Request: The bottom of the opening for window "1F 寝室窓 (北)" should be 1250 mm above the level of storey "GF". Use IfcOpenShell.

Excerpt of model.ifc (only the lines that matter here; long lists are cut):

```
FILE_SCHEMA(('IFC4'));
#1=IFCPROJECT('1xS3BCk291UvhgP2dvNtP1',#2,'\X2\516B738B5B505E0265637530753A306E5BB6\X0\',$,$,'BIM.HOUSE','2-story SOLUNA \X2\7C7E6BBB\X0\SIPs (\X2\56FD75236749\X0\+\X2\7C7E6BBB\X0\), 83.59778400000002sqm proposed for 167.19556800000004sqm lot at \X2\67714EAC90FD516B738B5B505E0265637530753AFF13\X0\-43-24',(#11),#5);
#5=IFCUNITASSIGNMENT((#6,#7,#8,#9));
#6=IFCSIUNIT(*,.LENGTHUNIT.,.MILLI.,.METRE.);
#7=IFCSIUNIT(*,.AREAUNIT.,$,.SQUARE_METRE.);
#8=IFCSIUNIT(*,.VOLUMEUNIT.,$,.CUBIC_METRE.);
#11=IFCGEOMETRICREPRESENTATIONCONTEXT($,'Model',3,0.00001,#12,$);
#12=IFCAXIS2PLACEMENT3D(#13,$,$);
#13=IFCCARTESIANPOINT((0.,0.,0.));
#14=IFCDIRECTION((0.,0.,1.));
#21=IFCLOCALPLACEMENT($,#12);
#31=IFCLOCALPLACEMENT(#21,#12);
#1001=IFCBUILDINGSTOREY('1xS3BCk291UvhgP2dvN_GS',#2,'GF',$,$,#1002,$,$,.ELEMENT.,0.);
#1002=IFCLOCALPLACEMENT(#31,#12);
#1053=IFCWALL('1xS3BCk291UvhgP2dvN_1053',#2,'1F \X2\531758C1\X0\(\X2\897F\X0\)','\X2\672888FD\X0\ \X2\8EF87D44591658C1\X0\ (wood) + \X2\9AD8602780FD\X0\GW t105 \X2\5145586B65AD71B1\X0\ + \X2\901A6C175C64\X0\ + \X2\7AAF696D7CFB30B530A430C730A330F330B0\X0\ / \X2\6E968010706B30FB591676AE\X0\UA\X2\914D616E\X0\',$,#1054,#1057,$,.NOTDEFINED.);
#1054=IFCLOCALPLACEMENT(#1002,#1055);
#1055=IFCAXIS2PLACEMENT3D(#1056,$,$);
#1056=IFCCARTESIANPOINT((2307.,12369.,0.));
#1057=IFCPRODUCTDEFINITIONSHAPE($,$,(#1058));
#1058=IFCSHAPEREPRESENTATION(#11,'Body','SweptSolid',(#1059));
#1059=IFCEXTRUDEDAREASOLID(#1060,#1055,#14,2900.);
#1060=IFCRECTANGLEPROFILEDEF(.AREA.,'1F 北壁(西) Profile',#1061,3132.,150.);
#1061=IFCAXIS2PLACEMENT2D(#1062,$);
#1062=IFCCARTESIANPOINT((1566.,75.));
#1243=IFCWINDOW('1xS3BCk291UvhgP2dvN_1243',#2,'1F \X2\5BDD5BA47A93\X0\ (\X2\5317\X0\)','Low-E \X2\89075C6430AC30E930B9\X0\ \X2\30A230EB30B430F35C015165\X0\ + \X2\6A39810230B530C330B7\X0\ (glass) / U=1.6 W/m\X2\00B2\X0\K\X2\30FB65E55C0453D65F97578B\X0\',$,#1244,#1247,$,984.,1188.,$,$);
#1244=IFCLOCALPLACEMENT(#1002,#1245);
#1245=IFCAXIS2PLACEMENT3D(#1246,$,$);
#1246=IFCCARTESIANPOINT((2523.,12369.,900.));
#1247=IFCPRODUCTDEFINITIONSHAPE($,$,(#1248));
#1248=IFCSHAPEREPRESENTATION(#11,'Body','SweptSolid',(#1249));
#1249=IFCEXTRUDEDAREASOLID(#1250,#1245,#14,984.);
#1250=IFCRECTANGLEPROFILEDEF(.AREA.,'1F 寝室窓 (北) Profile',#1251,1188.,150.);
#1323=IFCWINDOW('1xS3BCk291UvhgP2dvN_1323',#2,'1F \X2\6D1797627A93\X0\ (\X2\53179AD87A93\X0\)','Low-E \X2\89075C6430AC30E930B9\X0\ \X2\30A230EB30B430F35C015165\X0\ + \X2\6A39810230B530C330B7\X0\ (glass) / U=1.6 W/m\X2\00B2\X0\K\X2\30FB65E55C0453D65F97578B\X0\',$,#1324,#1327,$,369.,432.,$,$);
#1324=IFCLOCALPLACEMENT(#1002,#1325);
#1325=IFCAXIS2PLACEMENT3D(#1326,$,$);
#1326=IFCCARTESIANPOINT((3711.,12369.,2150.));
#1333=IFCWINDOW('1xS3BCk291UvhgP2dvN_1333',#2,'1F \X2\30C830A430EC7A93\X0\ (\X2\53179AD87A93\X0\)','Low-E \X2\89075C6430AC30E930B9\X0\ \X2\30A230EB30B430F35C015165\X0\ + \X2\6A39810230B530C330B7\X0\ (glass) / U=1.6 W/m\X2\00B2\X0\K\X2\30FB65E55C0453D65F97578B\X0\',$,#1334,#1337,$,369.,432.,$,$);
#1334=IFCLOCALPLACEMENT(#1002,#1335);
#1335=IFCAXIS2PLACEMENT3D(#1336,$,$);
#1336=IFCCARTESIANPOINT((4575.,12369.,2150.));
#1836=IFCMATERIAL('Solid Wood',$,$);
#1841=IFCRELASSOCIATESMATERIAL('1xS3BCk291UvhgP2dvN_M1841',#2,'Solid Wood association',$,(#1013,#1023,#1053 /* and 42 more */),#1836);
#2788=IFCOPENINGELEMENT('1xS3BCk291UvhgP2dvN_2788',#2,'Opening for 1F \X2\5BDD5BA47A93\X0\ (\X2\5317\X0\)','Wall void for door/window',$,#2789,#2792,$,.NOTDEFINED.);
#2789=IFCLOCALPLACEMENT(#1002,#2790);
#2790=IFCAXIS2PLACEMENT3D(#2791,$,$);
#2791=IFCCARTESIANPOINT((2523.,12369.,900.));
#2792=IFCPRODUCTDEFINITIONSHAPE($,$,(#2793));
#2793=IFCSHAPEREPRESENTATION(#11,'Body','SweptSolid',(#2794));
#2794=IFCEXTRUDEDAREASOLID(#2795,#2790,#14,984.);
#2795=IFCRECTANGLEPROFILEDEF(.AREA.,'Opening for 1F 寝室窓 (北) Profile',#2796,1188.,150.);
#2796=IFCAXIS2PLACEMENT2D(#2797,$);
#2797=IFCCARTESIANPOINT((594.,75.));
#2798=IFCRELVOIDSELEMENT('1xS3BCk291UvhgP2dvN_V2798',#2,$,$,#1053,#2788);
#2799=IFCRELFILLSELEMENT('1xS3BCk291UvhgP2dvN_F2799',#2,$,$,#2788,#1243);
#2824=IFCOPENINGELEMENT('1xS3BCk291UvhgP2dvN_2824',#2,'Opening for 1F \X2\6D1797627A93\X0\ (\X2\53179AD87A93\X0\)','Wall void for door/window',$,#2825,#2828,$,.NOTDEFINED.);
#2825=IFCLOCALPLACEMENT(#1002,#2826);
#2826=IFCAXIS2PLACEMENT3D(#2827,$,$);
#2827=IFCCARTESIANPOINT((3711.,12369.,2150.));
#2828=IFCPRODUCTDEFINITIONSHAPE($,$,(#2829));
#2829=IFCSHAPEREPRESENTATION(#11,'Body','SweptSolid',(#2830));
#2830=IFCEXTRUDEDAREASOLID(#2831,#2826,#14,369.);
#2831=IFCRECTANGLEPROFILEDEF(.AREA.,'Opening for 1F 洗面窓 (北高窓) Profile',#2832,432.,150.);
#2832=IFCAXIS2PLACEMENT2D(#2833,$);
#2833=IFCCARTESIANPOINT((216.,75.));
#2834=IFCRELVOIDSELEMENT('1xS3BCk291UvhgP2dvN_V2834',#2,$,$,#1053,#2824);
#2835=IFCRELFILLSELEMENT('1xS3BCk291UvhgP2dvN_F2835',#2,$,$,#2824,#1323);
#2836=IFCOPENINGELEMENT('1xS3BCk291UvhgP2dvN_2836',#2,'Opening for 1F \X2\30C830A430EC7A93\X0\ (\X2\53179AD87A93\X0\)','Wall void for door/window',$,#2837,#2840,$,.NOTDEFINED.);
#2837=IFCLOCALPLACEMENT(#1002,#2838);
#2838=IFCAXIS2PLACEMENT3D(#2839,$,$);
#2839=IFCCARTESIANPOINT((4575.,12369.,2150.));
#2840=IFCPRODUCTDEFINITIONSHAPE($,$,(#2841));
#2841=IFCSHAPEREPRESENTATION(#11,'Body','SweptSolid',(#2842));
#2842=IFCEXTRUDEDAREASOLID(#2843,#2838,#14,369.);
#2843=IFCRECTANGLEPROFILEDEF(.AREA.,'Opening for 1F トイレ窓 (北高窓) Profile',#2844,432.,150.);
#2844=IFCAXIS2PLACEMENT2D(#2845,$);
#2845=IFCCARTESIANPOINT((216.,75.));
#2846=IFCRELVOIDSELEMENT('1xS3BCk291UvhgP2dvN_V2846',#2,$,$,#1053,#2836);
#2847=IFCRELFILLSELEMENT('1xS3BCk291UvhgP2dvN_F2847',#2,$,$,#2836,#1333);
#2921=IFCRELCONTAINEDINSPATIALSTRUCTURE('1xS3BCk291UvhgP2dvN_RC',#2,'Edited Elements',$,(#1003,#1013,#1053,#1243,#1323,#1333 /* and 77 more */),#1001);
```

```python
import numpy as np
import ifcopenshell
import ifcopenshell.api.geometry
import ifcopenshell.geom
import ifcopenshell.util.element
import ifcopenshell.util.placement
import ifcopenshell.util.shape
import ifcopenshell.util.unit

model = ifcopenshell.open("model.ifc")
unit_scale = ifcopenshell.util.unit.calculate_unit_scale(model)

window = model.by_id(1243)
opening = window.FillsVoids[0].RelatingOpeningElement
storey = ifcopenshell.util.element.get_container(window, ifc_class="IfcBuildingStorey")
level = ifcopenshell.util.placement.get_local_placement(storey.ObjectPlacement)[2, 3]

# The opening's origin need not be at the sill, so measure its lowest point.
shape = ifcopenshell.geom.create_shape(ifcopenshell.geom.settings(), opening)
bottom = ifcopenshell.util.shape.get_shape_bottom_elevation(shape, shape.geometry) / unit_scale
dz = level + 1.25 / unit_scale - bottom

shift = np.array([0.0, 0.0, dz])
# The window is not placed relative to its opening, so move both.
for product in (opening, window):
    matrix = ifcopenshell.util.placement.get_local_placement(product.ObjectPlacement)
    matrix[:3, 3] += shift
    ifcopenshell.api.geometry.edit_object_placement(model, product=product, matrix=matrix, is_si=False)

print(f"moved by {dz * unit_scale:+.3f} m")

model.write("model_v2.ifc")
```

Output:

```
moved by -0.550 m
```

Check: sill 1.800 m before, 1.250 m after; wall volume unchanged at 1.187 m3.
